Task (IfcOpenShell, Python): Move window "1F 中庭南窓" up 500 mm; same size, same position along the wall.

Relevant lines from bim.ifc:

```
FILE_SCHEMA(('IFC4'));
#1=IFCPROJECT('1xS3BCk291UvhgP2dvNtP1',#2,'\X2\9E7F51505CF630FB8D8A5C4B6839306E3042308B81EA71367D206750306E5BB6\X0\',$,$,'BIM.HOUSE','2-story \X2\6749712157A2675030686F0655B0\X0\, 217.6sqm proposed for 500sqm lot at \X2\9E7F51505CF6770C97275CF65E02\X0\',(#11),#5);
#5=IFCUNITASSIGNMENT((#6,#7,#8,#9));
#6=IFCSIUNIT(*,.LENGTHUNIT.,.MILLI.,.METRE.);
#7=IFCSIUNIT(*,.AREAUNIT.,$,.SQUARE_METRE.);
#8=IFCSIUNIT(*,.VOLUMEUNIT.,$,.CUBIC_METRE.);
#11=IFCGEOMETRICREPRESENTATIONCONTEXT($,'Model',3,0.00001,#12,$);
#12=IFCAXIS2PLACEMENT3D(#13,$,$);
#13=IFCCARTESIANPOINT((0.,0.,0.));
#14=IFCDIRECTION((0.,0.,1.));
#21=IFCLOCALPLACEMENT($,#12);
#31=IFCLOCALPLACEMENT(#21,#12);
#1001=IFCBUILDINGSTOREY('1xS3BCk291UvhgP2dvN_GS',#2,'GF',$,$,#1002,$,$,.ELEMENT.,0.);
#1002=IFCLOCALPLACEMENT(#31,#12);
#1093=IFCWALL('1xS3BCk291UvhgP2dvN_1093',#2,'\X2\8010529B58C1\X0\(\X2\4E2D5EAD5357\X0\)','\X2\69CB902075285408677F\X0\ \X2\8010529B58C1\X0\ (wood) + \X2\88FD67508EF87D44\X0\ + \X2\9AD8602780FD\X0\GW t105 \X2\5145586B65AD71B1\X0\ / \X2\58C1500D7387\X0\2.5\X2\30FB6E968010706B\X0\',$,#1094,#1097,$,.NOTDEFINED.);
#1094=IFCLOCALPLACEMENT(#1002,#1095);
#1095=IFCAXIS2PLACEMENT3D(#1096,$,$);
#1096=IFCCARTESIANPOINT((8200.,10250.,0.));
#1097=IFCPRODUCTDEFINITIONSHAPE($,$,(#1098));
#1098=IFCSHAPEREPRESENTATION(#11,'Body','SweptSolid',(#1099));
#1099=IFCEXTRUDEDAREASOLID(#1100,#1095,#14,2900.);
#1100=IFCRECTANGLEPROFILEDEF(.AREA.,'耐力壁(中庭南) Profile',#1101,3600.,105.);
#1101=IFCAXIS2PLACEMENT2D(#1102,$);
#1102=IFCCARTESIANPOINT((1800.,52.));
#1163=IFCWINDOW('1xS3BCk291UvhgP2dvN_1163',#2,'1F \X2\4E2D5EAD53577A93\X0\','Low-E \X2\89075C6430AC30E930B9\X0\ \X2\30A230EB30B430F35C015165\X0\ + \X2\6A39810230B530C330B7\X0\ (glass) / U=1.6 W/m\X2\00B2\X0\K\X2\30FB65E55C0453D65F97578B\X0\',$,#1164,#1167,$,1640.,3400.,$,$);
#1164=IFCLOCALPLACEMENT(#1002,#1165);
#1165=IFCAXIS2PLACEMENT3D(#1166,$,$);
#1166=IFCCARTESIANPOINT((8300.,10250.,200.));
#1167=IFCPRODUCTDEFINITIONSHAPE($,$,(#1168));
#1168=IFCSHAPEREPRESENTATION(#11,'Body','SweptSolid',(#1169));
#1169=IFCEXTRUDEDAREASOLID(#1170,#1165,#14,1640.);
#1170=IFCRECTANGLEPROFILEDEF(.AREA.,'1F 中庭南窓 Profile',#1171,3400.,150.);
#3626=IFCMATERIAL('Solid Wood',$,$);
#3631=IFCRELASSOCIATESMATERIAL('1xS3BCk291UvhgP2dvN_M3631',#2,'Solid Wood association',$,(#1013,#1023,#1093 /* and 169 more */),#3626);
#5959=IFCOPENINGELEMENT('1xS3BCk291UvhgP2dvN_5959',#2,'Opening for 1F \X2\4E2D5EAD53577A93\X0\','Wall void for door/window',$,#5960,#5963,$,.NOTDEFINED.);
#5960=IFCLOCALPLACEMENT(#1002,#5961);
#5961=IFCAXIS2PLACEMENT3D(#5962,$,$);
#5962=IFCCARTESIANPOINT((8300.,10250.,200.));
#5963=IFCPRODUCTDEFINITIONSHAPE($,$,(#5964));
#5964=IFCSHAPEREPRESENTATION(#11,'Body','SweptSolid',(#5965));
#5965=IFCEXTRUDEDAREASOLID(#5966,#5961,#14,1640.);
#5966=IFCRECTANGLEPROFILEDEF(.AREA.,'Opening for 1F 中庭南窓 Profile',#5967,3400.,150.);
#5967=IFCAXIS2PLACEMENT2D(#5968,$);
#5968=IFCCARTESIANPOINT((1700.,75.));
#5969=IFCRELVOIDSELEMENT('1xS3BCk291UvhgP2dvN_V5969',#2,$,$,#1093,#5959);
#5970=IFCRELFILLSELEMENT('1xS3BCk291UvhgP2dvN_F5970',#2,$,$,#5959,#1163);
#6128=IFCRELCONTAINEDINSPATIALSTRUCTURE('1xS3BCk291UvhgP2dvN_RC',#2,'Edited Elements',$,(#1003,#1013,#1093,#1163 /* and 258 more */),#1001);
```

```python
import numpy as np
import ifcopenshell
import ifcopenshell.api.geometry
import ifcopenshell.util.placement
import ifcopenshell.util.unit

model = ifcopenshell.open("bim.ifc")
unit_scale = ifcopenshell.util.unit.calculate_unit_scale(model)

window = model.by_guid("1xS3BCk291UvhgP2dvN_1163")
opening = window.FillsVoids[0].RelatingOpeningElement
dz = 0.5 / unit_scale

shift = np.array([0.0, 0.0, dz])
# The window is not placed relative to its opening, so move both.
for product in (opening, window):
    matrix = ifcopenshell.util.placement.get_local_placement(product.ObjectPlacement)
    matrix[:3, 3] += shift
    ifcopenshell.api.geometry.edit_object_placement(model, product=product, matrix=matrix, is_si=False)

print(f"moved by {dz * unit_scale:+.3f} m")

model.write("bim_v2.ifc")
```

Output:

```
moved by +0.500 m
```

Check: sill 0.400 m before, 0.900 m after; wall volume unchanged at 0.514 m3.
